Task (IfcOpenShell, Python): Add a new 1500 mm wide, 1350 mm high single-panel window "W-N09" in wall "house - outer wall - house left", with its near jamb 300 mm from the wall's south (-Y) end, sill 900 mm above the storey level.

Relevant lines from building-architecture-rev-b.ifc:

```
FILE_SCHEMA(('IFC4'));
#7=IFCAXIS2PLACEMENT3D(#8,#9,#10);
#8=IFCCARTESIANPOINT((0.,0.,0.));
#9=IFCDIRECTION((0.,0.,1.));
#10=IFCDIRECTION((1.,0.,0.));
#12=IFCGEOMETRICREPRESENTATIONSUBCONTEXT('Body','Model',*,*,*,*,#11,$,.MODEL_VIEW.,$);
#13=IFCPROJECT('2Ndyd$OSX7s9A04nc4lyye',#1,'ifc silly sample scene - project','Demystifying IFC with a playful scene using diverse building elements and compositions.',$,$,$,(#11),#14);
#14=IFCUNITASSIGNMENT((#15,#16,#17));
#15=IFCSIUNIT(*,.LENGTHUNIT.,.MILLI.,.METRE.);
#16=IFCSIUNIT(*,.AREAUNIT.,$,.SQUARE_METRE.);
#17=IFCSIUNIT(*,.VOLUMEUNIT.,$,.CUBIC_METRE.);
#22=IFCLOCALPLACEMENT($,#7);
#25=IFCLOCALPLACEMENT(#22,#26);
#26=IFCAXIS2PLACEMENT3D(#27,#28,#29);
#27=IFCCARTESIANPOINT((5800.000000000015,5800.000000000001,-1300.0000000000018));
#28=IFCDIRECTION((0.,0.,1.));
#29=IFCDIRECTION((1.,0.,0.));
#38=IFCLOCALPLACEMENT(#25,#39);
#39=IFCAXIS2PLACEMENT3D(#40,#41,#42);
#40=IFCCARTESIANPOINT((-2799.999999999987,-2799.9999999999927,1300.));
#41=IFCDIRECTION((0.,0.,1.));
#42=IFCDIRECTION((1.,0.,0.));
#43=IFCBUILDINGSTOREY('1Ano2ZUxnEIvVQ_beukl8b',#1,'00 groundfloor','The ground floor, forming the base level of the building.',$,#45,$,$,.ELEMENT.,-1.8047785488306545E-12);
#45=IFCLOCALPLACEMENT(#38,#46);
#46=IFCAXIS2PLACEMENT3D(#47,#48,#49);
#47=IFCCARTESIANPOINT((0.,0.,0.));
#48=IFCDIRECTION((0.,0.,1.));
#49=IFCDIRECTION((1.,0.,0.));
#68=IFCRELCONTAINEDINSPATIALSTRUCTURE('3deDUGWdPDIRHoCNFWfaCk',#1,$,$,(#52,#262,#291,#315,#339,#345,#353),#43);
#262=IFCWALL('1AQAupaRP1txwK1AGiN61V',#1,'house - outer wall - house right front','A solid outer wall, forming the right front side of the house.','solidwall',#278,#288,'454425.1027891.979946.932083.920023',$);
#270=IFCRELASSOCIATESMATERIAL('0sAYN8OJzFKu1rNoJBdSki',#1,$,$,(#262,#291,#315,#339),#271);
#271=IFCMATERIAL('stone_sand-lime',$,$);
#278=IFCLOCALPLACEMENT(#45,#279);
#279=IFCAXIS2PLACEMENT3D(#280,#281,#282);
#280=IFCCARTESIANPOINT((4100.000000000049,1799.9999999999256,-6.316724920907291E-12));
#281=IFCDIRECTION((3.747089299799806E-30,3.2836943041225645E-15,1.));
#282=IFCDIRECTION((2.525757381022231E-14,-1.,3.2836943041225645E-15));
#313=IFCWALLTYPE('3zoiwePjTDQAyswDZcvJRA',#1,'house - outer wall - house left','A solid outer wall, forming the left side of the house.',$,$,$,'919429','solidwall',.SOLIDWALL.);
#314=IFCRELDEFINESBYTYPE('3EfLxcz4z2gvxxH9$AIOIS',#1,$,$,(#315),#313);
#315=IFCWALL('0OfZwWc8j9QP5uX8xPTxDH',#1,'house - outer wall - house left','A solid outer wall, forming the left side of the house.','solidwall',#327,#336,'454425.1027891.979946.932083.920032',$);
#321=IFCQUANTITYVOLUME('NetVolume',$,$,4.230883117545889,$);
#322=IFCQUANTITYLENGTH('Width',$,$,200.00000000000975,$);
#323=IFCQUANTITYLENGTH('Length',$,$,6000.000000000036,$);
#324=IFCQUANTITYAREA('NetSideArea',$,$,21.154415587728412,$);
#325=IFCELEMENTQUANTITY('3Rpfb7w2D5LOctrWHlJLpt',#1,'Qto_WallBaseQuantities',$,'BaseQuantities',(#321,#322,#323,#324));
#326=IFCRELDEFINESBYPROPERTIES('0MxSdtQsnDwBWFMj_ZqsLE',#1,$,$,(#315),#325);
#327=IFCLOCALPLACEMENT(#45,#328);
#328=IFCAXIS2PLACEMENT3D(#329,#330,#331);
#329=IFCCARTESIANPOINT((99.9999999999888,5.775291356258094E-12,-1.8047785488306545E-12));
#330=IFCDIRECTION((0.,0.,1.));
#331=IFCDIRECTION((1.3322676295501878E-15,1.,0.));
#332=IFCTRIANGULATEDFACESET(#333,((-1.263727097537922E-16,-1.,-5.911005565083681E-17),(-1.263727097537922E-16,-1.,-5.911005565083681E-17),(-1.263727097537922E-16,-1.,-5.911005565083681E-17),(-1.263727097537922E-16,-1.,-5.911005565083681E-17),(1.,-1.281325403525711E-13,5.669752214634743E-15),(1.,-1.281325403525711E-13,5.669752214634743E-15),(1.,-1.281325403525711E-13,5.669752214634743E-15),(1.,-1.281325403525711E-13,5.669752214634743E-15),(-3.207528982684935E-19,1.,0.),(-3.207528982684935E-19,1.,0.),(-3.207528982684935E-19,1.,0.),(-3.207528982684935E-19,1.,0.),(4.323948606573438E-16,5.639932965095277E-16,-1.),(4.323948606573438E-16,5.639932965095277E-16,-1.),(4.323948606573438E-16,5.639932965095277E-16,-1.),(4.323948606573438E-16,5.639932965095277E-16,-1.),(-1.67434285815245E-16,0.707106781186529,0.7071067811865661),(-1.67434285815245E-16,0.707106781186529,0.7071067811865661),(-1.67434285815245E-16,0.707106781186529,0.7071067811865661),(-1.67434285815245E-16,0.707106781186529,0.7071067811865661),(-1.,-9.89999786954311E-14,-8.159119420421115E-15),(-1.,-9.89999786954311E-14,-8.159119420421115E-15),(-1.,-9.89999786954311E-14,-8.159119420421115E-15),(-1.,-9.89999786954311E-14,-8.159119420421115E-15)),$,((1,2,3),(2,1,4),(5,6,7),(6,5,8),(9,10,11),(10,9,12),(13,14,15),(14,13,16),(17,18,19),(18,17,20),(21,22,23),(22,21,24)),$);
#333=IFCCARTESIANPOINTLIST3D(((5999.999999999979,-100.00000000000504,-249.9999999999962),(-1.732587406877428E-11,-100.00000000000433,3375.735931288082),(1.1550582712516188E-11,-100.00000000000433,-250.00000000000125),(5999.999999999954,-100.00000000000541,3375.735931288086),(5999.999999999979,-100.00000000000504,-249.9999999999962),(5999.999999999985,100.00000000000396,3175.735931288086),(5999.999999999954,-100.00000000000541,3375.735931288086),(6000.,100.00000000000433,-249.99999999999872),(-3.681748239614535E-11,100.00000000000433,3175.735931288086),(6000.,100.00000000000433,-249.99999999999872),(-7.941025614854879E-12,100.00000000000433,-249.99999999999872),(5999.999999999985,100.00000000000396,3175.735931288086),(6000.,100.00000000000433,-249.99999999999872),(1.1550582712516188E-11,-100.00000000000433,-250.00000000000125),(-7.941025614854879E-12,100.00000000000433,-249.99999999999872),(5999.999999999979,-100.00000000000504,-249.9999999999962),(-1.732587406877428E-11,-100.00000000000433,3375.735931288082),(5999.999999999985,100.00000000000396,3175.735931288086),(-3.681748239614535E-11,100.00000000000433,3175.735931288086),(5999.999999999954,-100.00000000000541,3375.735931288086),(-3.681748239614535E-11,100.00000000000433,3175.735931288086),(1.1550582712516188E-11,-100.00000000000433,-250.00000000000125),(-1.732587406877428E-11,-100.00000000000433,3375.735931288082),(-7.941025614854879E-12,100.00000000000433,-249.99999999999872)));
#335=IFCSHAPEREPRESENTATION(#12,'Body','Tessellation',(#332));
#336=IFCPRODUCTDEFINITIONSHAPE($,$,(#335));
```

```python
import numpy as np
import ifcopenshell
import ifcopenshell.api.feature
import ifcopenshell.api.geometry
import ifcopenshell.api.pset
import ifcopenshell.api.root
import ifcopenshell.api.spatial
import ifcopenshell.geom
import ifcopenshell.util.element
import ifcopenshell.util.placement
import ifcopenshell.util.representation
import ifcopenshell.util.shape
import ifcopenshell.util.unit

model = ifcopenshell.open("building-architecture-rev-b.ifc")
unit_scale = ifcopenshell.util.unit.calculate_unit_scale(model)
area_scale = ifcopenshell.util.unit.calculate_unit_scale(model, "AREAUNIT")
volume_scale = ifcopenshell.util.unit.calculate_unit_scale(model, "VOLUMEUNIT")
settings = ifcopenshell.geom.settings()


def volume(element):
    """Net volume in cubic metres, openings subtracted."""
    shape = ifcopenshell.geom.create_shape(settings, element)
    return ifcopenshell.util.shape.get_volume(shape.geometry)


wall = model.by_guid("0OfZwWc8j9QP5uX8xPTxDH")
storey = ifcopenshell.util.element.get_container(wall, ifc_class="IfcBuildingStorey")
context = ifcopenshell.util.representation.get_context(model, "Model", "Body", "MODEL_VIEW")
before = volume(wall)

width, height, from_end, sill = 1.5, 1.35, 0.3, 0.9  # metres

# The wall runs along its own X axis, and the end named is its -X end.
wall_shape = ifcopenshell.geom.create_shape(settings, wall)
x, y, z = ifcopenshell.util.shape.get_vertices(wall_shape.geometry).T
start = x.min() + from_end
face, thickness = float(y.min()), float(y.max() - y.min())
wall_matrix = ifcopenshell.util.placement.get_local_placement(wall.ObjectPlacement)
level = ifcopenshell.util.placement.get_local_placement(storey.ObjectPlacement)[2, 3]


def in_wall(x, y):
    """Placement at x, y metres in the wall's axes, at sill height."""
    matrix = wall_matrix.copy()
    matrix[:, 3] = wall_matrix @ np.array([x / unit_scale, y / unit_scale, 0.0, 1.0])
    matrix[2, 3] = level + sill / unit_scale
    return matrix


# Opening: a box that overshoots both wall faces by 50 mm.
opening = ifcopenshell.api.root.create_entity(model, ifc_class="IfcOpeningElement", predefined_type="OPENING")
box = ifcopenshell.api.geometry.add_wall_representation(
    model, context=context, length=width, height=height, thickness=thickness + 0.1
)
ifcopenshell.api.geometry.assign_representation(model, product=opening, representation=box)
ifcopenshell.api.geometry.edit_object_placement(model, product=opening, matrix=in_wall(start, face - 0.05), is_si=False)
ifcopenshell.api.feature.add_feature(model, feature=opening, element=wall)

window = ifcopenshell.api.root.create_entity(model, ifc_class="IfcWindow", name="W-N09", predefined_type="WINDOW")
window.OverallWidth, window.OverallHeight = width / unit_scale, height / unit_scale
window.PartitioningType = "SINGLE_PANEL"
body = ifcopenshell.api.geometry.add_window_representation(
    model,
    context=context,
    overall_width=window.OverallWidth,
    overall_height=window.OverallHeight,
    partition_type="SINGLE_PANEL",
)
ifcopenshell.api.geometry.assign_representation(model, product=window, representation=body)
ifcopenshell.api.spatial.assign_container(model, products=[window], relating_structure=storey)
ifcopenshell.api.feature.add_filling(model, opening=opening, element=window)

# Centre the window in the wall's thickness.
ifcopenshell.api.geometry.edit_object_placement(model, product=window, matrix=in_wall(start, face), is_si=False)
window_shape = ifcopenshell.geom.create_shape(settings, window)
depth = ifcopenshell.util.shape.get_vertices(window_shape.geometry)[:, 1]
offset = face + thickness / 2 - (depth.min() + depth.max()) / 2
ifcopenshell.api.geometry.edit_object_placement(model, product=window, matrix=in_wall(start, offset), is_si=False)

after = volume(wall)

# Update the wall's stored quantities.
qto = model.by_id(ifcopenshell.util.element.get_pset(wall, "Qto_WallBaseQuantities", should_inherit=False)["id"])
ifcopenshell.api.pset.edit_qto(model, qto=qto, properties={
    "NetVolume": after / volume_scale,
    "NetSideArea": after / thickness / area_scale,
})

print(f"wall volume {before:.3f} -> {after:.3f} m3")

model.write("building-architecture-rev-b_updated.ifc")
```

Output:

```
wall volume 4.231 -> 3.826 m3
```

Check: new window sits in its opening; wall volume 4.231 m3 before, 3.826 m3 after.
